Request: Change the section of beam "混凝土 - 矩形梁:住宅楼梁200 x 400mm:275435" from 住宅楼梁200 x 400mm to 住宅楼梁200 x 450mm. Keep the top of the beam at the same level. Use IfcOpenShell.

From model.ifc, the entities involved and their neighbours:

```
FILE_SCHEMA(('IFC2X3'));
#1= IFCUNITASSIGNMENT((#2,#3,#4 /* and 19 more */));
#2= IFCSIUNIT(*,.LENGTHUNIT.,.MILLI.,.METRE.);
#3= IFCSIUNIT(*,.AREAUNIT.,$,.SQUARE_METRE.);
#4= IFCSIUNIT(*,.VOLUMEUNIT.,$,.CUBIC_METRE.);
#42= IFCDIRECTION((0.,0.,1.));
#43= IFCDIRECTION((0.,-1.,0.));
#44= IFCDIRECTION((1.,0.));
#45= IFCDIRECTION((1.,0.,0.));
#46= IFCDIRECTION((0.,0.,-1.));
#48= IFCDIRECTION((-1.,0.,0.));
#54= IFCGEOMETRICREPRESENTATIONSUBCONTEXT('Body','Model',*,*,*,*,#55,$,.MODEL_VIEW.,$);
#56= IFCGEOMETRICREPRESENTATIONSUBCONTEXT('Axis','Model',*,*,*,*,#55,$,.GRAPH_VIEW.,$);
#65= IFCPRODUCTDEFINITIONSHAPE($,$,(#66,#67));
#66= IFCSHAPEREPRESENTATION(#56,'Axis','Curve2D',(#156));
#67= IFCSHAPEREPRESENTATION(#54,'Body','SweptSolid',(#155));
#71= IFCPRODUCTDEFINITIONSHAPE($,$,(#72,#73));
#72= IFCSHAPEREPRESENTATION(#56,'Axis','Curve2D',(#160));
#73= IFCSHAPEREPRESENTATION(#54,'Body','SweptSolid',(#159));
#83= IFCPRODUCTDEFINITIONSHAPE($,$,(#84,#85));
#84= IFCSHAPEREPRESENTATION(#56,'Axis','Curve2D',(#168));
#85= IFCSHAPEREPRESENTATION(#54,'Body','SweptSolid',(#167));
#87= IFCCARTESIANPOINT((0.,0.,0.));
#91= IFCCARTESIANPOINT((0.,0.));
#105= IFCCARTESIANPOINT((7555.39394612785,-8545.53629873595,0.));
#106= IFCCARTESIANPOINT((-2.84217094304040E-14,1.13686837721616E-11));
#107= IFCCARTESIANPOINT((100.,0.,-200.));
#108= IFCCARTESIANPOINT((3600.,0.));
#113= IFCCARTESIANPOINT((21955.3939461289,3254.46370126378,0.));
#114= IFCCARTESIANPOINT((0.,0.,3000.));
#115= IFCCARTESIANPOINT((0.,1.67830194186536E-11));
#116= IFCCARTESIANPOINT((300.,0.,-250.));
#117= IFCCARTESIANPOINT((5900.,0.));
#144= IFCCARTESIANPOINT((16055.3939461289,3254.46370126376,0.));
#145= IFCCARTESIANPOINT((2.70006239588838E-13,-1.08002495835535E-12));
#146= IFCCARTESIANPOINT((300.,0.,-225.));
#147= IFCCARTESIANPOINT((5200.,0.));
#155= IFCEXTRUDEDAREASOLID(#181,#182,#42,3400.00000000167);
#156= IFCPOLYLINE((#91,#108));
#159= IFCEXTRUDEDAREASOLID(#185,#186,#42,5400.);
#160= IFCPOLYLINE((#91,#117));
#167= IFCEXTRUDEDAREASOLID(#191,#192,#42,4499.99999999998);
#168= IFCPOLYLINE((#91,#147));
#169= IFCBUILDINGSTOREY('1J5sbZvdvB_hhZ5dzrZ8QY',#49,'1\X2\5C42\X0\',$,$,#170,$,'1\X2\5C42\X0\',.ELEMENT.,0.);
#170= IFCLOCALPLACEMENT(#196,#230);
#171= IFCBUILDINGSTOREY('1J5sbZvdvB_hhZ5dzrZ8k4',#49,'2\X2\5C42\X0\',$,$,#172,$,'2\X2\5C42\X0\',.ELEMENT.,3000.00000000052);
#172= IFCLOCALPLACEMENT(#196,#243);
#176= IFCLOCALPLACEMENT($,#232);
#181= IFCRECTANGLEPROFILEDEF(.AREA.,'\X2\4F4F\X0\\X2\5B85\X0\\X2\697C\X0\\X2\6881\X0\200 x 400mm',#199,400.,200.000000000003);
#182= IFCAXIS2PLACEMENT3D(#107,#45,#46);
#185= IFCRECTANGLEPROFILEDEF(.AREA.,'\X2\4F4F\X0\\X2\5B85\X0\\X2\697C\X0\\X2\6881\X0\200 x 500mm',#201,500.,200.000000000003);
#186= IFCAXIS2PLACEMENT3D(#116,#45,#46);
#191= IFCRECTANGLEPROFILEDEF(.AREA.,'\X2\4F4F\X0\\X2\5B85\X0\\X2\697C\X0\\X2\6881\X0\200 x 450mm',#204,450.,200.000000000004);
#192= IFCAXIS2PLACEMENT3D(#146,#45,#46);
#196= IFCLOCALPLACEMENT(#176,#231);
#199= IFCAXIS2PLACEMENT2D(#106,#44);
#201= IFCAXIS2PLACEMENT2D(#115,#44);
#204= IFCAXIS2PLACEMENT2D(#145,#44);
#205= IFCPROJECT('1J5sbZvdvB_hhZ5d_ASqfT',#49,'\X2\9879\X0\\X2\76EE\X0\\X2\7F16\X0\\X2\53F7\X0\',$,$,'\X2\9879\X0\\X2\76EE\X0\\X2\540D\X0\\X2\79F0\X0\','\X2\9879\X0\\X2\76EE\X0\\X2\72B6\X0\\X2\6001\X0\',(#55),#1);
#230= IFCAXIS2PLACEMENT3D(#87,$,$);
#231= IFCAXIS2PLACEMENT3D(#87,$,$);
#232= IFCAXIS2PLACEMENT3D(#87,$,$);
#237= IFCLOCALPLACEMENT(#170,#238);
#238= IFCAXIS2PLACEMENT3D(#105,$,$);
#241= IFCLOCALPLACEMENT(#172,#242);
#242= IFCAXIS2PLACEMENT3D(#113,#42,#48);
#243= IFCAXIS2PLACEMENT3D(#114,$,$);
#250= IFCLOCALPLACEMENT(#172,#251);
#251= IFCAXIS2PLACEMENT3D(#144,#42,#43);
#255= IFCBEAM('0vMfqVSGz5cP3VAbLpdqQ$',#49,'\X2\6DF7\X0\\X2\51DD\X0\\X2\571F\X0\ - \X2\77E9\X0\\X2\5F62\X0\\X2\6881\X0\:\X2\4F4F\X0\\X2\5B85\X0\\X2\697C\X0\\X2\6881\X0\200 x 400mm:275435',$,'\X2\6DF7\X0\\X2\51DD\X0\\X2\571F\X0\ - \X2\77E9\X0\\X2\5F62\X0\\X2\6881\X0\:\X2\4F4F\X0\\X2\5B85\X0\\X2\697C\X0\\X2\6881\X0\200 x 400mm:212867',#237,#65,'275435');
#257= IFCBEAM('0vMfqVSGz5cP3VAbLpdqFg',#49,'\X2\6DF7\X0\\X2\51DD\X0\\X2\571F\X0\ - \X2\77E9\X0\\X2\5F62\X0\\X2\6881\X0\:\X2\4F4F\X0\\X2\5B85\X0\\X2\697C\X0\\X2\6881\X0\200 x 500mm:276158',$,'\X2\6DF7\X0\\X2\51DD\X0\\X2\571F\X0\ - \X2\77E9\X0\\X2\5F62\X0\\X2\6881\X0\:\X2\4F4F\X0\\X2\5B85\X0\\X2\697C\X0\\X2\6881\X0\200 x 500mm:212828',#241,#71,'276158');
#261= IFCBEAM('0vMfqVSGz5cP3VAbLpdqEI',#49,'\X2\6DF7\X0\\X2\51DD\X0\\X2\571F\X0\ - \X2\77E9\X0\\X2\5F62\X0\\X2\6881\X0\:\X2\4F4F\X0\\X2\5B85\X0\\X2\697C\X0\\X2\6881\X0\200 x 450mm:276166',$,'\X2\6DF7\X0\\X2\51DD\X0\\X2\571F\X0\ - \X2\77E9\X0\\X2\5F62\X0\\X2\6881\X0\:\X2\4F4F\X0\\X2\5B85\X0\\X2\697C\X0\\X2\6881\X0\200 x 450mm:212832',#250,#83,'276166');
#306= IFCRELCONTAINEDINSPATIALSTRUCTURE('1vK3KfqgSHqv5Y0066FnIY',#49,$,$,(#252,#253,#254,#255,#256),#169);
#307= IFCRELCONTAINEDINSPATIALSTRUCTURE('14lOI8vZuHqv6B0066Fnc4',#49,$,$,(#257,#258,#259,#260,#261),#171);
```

```python
import ifcopenshell
import ifcopenshell.util.element
import ifcopenshell.util.representation

model = ifcopenshell.open("model.ifc")

member = model.by_guid("0vMfqVSGz5cP3VAbLpdqQ$")
source = next(p for p in model.by_type("IfcRectangleProfileDef") if p.ProfileName == "住宅楼梁200 x 450mm")

body = ifcopenshell.util.representation.get_representation(member, "Model", "Body")
solid = body.Items[0]
old_profile = solid.SweptArea

# Copy the section's sizes but keep this member's own profile position.
profile = ifcopenshell.util.element.copy(model, source)
# Profiles are centred, so shift by half the change in depth to hold the top.
shift = (old_profile.XDim - profile.XDim) / 2
x, y = old_profile.Position.Location.Coordinates
up = (-1.0, 0.0)  # upwards, in the solid's own plane
location = model.createIfcCartesianPoint((x + up[0] * shift, y + up[1] * shift))
profile.Position = model.createIfcAxis2Placement2D(location, old_profile.Position.RefDirection)
solid.SweptArea = profile
if not model.get_total_inverses(old_profile):
    ifcopenshell.util.element.remove_deep2(model, old_profile)
member.Name = member.Name.replace("住宅楼梁200 x 400mm", "住宅楼梁200 x 450mm")
member.ObjectType = member.ObjectType.replace("住宅楼梁200 x 400mm", "住宅楼梁200 x 450mm")

print(solid.SweptArea)

model.write("model_edited.ifc")
```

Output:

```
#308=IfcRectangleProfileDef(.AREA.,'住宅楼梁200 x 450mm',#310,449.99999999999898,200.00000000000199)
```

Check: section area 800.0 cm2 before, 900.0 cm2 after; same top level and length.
